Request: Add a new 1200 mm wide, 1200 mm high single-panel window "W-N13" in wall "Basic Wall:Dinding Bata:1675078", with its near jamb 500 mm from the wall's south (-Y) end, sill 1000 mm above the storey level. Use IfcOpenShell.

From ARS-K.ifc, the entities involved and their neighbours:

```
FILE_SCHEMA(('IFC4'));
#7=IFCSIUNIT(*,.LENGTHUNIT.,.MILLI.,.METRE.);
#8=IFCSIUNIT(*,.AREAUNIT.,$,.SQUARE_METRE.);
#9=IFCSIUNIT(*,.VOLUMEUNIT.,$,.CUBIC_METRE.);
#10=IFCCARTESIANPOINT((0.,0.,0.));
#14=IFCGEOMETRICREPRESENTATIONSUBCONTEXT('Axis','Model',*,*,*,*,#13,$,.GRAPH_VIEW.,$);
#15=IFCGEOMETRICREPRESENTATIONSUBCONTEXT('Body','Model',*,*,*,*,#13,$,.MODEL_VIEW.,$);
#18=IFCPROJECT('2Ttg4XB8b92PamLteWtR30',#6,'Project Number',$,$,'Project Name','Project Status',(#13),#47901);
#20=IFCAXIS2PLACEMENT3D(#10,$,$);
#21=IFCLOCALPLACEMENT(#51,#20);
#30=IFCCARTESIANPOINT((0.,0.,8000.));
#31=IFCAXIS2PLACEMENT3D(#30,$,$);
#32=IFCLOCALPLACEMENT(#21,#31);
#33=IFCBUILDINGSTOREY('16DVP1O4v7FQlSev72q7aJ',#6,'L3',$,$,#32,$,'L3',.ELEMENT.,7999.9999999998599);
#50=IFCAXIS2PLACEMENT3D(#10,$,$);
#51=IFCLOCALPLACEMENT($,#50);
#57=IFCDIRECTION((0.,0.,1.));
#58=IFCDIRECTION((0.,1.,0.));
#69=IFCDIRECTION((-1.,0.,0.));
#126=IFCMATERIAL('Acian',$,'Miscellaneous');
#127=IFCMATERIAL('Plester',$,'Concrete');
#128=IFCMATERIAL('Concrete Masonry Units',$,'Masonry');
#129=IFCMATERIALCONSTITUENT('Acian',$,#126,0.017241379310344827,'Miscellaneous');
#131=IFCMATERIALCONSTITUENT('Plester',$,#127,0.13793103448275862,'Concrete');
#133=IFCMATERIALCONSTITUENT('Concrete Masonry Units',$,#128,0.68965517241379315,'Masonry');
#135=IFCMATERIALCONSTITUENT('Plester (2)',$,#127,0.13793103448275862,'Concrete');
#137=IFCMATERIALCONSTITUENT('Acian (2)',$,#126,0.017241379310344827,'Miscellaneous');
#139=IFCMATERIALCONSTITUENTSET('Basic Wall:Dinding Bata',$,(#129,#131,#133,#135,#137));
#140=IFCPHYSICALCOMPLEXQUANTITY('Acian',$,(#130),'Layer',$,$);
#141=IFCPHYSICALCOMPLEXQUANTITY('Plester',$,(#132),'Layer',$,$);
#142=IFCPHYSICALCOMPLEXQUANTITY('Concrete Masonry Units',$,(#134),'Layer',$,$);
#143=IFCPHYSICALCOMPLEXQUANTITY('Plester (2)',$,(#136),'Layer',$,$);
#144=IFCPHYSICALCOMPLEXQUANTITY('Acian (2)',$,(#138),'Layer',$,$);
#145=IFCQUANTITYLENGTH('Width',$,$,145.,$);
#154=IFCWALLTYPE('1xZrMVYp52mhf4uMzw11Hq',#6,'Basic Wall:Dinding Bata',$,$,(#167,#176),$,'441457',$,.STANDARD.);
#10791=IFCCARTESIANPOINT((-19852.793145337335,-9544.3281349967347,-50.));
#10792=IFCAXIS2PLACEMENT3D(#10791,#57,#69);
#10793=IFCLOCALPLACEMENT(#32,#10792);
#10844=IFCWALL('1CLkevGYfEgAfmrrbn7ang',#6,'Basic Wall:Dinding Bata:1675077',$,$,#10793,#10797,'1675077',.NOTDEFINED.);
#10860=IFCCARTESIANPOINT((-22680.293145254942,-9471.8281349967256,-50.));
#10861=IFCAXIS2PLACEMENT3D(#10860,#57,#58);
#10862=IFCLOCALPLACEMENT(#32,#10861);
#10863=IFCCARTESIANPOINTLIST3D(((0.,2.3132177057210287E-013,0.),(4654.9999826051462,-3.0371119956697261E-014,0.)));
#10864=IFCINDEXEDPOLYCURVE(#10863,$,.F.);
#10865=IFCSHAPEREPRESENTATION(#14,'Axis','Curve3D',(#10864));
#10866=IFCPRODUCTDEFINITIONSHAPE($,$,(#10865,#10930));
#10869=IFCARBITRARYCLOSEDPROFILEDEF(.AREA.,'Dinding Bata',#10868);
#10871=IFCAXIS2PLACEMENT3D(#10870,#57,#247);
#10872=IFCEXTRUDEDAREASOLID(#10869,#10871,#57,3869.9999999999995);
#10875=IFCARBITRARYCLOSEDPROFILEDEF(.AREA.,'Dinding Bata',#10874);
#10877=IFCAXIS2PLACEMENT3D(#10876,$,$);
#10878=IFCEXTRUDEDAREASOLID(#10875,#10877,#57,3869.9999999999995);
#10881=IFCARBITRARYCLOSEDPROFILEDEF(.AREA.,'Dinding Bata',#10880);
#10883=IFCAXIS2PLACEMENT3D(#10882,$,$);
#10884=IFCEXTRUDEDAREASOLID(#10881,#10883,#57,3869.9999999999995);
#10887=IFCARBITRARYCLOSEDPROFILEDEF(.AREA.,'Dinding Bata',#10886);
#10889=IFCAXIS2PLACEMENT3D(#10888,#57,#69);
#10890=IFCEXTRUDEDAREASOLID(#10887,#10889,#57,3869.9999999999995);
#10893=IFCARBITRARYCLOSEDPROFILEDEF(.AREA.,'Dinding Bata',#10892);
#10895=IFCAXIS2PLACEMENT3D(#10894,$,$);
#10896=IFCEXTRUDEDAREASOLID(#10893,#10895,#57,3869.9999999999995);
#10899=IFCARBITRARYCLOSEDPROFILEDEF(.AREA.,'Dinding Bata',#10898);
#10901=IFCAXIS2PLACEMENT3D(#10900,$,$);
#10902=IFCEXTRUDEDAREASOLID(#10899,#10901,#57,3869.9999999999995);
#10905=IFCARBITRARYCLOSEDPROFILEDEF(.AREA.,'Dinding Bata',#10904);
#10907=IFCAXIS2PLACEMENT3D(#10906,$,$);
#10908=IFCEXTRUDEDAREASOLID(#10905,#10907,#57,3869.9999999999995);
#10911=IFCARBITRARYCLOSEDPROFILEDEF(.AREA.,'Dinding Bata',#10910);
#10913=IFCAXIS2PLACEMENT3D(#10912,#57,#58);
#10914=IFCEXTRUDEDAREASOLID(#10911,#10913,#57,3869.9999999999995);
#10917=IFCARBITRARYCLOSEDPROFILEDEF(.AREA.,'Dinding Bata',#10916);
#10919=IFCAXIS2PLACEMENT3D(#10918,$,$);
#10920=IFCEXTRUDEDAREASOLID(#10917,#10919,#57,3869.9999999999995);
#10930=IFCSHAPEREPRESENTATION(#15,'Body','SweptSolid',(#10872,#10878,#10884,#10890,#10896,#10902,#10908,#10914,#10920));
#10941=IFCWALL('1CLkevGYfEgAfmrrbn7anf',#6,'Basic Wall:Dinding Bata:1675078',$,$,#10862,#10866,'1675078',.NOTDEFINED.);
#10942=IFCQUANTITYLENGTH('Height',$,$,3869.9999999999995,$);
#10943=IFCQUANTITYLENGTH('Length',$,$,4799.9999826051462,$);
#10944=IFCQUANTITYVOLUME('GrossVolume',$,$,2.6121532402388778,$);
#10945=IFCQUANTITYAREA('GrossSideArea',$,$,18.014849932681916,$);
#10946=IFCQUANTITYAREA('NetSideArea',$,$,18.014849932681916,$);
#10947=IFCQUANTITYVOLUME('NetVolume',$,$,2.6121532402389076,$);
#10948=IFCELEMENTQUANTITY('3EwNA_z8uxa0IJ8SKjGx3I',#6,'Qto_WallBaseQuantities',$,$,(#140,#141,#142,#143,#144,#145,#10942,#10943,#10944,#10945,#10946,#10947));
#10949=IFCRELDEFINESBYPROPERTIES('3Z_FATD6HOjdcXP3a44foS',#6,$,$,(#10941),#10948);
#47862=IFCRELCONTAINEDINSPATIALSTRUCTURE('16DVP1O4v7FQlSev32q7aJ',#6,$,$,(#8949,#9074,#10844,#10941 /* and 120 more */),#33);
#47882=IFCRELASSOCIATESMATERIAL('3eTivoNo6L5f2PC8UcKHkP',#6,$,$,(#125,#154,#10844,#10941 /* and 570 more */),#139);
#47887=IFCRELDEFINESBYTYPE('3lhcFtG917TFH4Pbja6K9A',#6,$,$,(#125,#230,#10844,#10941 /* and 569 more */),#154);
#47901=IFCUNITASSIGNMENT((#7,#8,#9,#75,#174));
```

```python
import numpy as np
import ifcopenshell
import ifcopenshell.api.feature
import ifcopenshell.api.geometry
import ifcopenshell.api.pset
import ifcopenshell.api.root
import ifcopenshell.api.spatial
import ifcopenshell.geom
import ifcopenshell.util.element
import ifcopenshell.util.placement
import ifcopenshell.util.representation
import ifcopenshell.util.shape
import ifcopenshell.util.unit

model = ifcopenshell.open("ARS-K.ifc")
unit_scale = ifcopenshell.util.unit.calculate_unit_scale(model)
area_scale = ifcopenshell.util.unit.calculate_unit_scale(model, "AREAUNIT")
volume_scale = ifcopenshell.util.unit.calculate_unit_scale(model, "VOLUMEUNIT")
settings = ifcopenshell.geom.settings()


def volume(element):
    """Net volume in cubic metres, openings subtracted."""
    shape = ifcopenshell.geom.create_shape(settings, element)
    return ifcopenshell.util.shape.get_volume(shape.geometry)


wall = model.by_id(10941)
storey = ifcopenshell.util.element.get_container(wall, ifc_class="IfcBuildingStorey")
context = ifcopenshell.util.representation.get_context(model, "Model", "Body", "MODEL_VIEW")
before = volume(wall)

width, height, from_end, sill = 1.2, 1.2, 0.5, 1  # metres

# The wall runs along its own X axis, and the end named is its -X end.
wall_shape = ifcopenshell.geom.create_shape(settings, wall)
x, y, z = ifcopenshell.util.shape.get_vertices(wall_shape.geometry).T
start = x.min() + from_end
face, thickness = float(y.min()), float(y.max() - y.min())
wall_matrix = ifcopenshell.util.placement.get_local_placement(wall.ObjectPlacement)
level = ifcopenshell.util.placement.get_local_placement(storey.ObjectPlacement)[2, 3]


def in_wall(x, y):
    """Placement at x, y metres in the wall's axes, at sill height."""
    matrix = wall_matrix.copy()
    matrix[:, 3] = wall_matrix @ np.array([x / unit_scale, y / unit_scale, 0.0, 1.0])
    matrix[2, 3] = level + sill / unit_scale
    return matrix


# Opening: a box that overshoots both wall faces by 50 mm.
opening = ifcopenshell.api.root.create_entity(model, ifc_class="IfcOpeningElement", predefined_type="OPENING")
box = ifcopenshell.api.geometry.add_wall_representation(
    model, context=context, length=width, height=height, thickness=thickness + 0.1
)
ifcopenshell.api.geometry.assign_representation(model, product=opening, representation=box)
ifcopenshell.api.geometry.edit_object_placement(model, product=opening, matrix=in_wall(start, face - 0.05), is_si=False)
ifcopenshell.api.feature.add_feature(model, feature=opening, element=wall)

window = ifcopenshell.api.root.create_entity(model, ifc_class="IfcWindow", name="W-N13", predefined_type="WINDOW")
window.OverallWidth, window.OverallHeight = width / unit_scale, height / unit_scale
window.PartitioningType = "SINGLE_PANEL"
body = ifcopenshell.api.geometry.add_window_representation(
    model,
    context=context,
    overall_width=window.OverallWidth,
    overall_height=window.OverallHeight,
    partition_type="SINGLE_PANEL",
)
ifcopenshell.api.geometry.assign_representation(model, product=window, representation=body)
ifcopenshell.api.spatial.assign_container(model, products=[window], relating_structure=storey)
ifcopenshell.api.feature.add_filling(model, opening=opening, element=window)

# Centre the window in the wall's thickness.
ifcopenshell.api.geometry.edit_object_placement(model, product=window, matrix=in_wall(start, face), is_si=False)
window_shape = ifcopenshell.geom.create_shape(settings, window)
depth = ifcopenshell.util.shape.get_vertices(window_shape.geometry)[:, 1]
offset = face + thickness / 2 - (depth.min() + depth.max()) / 2
ifcopenshell.api.geometry.edit_object_placement(model, product=window, matrix=in_wall(start, offset), is_si=False)

after = volume(wall)

# Update the wall's stored quantities.
qto = model.by_id(ifcopenshell.util.element.get_pset(wall, "Qto_WallBaseQuantities", should_inherit=False)["id"])
ifcopenshell.api.pset.edit_qto(model, qto=qto, properties={
    "NetSideArea": after / thickness / area_scale,
    "NetVolume": after / volume_scale,
})

print(f"wall volume {before:.3f} -> {after:.3f} m3")

model.write("ARS-K_v2.ifc")
```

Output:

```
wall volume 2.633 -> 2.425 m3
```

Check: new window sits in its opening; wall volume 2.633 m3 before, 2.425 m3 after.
